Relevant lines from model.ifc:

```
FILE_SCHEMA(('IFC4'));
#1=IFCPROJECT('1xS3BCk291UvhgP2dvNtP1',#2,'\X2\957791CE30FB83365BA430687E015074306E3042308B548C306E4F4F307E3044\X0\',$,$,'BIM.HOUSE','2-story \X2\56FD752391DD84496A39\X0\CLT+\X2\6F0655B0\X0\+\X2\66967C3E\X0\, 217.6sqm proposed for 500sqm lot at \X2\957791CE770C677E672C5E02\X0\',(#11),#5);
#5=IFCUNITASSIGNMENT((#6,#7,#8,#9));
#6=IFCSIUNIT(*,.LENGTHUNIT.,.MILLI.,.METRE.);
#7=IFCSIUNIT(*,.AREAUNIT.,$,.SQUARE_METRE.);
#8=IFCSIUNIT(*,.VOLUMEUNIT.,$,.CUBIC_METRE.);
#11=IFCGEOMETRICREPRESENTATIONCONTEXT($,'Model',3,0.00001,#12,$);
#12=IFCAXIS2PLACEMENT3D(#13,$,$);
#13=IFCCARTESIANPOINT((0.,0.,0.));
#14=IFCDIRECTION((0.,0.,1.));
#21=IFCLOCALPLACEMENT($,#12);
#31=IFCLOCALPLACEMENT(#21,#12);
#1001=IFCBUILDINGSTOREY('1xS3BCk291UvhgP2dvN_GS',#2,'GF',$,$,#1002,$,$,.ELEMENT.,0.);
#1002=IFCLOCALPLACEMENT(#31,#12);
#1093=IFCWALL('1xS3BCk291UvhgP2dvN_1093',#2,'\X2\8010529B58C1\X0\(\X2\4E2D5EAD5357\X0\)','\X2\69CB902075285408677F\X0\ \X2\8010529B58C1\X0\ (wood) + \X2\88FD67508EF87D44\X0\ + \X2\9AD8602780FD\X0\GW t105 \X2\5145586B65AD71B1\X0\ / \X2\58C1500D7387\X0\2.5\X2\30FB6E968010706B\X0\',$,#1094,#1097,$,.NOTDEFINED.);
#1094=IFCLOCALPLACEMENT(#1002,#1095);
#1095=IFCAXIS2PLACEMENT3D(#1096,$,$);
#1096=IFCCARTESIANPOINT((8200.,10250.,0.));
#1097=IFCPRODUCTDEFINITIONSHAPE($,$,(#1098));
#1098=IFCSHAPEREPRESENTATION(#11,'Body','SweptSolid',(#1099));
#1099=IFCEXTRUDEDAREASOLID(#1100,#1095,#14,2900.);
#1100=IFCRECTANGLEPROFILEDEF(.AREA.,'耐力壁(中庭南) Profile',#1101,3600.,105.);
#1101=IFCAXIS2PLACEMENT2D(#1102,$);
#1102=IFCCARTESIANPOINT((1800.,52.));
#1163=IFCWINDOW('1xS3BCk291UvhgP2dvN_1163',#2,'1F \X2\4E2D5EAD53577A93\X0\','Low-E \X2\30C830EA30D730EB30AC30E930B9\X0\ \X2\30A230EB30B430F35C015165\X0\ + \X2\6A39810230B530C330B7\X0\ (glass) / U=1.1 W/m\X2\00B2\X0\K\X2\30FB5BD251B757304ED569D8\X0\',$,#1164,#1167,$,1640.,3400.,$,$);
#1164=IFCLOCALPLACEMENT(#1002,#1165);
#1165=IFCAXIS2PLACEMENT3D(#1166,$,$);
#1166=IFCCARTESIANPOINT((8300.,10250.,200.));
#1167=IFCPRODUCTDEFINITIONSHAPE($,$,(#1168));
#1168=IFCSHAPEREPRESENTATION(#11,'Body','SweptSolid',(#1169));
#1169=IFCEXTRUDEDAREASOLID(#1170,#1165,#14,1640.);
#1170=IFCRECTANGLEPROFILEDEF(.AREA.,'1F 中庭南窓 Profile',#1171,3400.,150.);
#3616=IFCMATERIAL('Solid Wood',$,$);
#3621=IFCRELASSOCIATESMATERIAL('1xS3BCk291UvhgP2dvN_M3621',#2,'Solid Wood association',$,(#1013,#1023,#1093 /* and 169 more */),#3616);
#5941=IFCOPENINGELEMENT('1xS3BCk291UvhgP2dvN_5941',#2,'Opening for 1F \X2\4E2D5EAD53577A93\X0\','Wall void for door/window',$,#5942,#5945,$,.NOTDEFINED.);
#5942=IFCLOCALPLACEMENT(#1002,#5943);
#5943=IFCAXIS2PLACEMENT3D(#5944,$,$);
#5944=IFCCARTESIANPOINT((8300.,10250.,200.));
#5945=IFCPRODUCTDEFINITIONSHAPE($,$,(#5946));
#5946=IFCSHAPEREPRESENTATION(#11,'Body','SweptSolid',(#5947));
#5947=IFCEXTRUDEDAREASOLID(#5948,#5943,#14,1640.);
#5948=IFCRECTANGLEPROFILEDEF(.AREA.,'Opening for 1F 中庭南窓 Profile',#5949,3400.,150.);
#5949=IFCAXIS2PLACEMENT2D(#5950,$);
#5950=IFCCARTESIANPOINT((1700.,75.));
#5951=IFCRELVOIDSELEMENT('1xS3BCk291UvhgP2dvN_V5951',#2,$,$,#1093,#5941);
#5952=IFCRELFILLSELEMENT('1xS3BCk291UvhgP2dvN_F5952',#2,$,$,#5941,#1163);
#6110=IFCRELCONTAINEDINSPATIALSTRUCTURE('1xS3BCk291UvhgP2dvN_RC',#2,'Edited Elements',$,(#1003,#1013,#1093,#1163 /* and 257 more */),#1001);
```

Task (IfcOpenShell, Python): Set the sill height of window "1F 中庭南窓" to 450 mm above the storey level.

```python
import numpy as np
import ifcopenshell
import ifcopenshell.api.geometry
import ifcopenshell.geom
import ifcopenshell.util.element
import ifcopenshell.util.placement
import ifcopenshell.util.shape
import ifcopenshell.util.unit

model = ifcopenshell.open("model.ifc")
unit_scale = ifcopenshell.util.unit.calculate_unit_scale(model)

window = model.by_guid("1xS3BCk291UvhgP2dvN_1163")
opening = window.FillsVoids[0].RelatingOpeningElement
storey = ifcopenshell.util.element.get_container(window, ifc_class="IfcBuildingStorey")
level = ifcopenshell.util.placement.get_local_placement(storey.ObjectPlacement)[2, 3]

# The opening's origin need not be at the sill, so measure its lowest point.
shape = ifcopenshell.geom.create_shape(ifcopenshell.geom.settings(), opening)
bottom = ifcopenshell.util.shape.get_shape_bottom_elevation(shape, shape.geometry) / unit_scale
dz = level + 0.45 / unit_scale - bottom

shift = np.array([0.0, 0.0, dz])
# The window is not placed relative to its opening, so move both.
for product in (opening, window):
    matrix = ifcopenshell.util.placement.get_local_placement(product.ObjectPlacement)
    matrix[:3, 3] += shift
    ifcopenshell.api.geometry.edit_object_placement(model, product=product, matrix=matrix, is_si=False)

print(f"moved by {dz * unit_scale:+.3f} m")

model.write("model_edited.ifc")
```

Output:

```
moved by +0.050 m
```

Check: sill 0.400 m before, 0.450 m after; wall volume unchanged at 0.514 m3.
